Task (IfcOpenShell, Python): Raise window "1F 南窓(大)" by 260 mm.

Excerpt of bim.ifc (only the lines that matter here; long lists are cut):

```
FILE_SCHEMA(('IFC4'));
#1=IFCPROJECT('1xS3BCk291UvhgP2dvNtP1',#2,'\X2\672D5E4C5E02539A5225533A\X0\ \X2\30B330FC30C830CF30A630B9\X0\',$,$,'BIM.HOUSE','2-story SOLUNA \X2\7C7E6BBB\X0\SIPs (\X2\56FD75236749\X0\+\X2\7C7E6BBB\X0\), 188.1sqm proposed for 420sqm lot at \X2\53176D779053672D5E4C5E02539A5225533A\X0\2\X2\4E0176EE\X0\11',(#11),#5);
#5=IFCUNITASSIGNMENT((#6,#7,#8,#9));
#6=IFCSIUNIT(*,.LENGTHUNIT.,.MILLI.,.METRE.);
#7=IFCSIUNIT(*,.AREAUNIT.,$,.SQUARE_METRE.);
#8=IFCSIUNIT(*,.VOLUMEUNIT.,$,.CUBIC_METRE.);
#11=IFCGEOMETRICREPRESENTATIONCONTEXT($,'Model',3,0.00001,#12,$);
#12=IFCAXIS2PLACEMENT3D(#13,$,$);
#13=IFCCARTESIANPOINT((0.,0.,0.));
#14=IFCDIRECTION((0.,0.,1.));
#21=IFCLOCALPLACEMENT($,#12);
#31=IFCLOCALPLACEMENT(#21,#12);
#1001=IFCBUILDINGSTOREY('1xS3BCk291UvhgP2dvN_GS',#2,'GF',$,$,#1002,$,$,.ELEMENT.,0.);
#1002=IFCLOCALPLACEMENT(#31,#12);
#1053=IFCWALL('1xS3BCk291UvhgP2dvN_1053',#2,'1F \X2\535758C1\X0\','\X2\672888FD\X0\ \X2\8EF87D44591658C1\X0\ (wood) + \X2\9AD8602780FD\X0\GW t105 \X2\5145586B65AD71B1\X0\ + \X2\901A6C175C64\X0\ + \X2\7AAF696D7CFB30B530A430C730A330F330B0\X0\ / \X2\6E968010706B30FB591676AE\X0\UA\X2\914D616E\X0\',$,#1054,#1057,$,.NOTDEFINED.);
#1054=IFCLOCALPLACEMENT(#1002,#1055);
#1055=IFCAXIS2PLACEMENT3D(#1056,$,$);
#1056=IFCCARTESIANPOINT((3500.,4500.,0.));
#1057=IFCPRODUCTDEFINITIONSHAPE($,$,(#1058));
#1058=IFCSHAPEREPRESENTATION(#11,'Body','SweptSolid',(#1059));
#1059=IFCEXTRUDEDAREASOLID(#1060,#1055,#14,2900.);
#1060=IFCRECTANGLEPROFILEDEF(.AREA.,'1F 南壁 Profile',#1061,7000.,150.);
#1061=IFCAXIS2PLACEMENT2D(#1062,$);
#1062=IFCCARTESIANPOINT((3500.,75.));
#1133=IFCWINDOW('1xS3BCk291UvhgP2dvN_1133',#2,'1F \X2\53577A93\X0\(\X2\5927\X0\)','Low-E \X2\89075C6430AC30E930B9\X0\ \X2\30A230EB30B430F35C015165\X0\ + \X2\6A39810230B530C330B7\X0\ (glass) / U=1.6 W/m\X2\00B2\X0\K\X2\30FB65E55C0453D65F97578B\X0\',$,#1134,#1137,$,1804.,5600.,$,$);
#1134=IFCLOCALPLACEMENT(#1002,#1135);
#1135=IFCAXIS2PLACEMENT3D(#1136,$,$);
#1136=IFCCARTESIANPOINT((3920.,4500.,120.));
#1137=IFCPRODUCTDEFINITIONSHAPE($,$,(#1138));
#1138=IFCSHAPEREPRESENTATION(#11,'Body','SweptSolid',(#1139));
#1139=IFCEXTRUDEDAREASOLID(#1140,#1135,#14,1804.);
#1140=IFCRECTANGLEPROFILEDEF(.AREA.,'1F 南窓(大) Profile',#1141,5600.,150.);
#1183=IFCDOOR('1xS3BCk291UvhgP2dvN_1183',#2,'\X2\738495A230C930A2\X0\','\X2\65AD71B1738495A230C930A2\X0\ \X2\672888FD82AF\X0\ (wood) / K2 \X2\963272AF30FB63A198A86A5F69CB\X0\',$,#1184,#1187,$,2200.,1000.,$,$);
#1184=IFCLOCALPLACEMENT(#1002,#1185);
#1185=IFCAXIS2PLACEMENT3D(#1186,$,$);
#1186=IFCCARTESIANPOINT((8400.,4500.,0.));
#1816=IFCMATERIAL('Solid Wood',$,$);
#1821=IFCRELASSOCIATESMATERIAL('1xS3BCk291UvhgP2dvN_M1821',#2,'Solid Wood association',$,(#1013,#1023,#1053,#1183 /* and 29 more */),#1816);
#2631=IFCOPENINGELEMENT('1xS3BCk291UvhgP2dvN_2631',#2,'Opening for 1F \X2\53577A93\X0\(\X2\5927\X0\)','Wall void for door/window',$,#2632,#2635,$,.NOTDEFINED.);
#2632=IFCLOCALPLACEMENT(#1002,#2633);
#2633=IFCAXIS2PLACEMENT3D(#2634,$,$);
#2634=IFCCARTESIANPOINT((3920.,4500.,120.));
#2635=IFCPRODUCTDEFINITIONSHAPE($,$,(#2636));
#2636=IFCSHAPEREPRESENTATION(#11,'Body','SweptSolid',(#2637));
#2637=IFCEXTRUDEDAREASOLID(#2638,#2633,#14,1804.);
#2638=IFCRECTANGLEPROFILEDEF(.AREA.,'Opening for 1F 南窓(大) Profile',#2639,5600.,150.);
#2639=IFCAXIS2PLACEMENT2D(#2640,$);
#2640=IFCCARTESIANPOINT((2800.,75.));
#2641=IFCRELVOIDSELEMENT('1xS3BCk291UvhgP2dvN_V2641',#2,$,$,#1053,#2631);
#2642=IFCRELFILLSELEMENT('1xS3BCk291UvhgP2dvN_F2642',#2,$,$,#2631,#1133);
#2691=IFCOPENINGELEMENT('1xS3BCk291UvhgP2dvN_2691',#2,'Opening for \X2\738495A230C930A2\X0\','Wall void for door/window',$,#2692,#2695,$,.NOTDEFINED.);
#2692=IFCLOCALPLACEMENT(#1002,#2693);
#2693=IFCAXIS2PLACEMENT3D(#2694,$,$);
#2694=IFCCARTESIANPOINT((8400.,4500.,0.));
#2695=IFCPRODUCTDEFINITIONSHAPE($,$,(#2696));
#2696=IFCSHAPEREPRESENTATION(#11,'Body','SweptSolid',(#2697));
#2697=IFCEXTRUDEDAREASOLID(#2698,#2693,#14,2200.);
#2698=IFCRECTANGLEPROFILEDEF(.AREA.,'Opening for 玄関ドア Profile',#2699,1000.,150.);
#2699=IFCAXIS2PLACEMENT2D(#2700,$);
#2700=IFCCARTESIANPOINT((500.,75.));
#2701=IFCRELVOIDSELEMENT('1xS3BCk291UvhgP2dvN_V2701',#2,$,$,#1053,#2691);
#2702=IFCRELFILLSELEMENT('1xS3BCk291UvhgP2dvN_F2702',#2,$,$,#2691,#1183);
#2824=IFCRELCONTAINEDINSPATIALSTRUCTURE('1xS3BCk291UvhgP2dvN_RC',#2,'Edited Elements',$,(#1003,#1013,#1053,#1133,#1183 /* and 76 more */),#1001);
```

```python
import numpy as np
import ifcopenshell
import ifcopenshell.api.geometry
import ifcopenshell.util.placement
import ifcopenshell.util.unit

model = ifcopenshell.open("bim.ifc")
unit_scale = ifcopenshell.util.unit.calculate_unit_scale(model)

window = model.by_guid("1xS3BCk291UvhgP2dvN_1133")
opening = window.FillsVoids[0].RelatingOpeningElement
dz = 0.26 / unit_scale

shift = np.array([0.0, 0.0, dz])
# The window is not placed relative to its opening, so move both.
for product in (opening, window):
    matrix = ifcopenshell.util.placement.get_local_placement(product.ObjectPlacement)
    matrix[:3, 3] += shift
    ifcopenshell.api.geometry.edit_object_placement(model, product=product, matrix=matrix, is_si=False)

print(f"moved by {dz * unit_scale:+.3f} m")

model.write("bim_v2.ifc")
```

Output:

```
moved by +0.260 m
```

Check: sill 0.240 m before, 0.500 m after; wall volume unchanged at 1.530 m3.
